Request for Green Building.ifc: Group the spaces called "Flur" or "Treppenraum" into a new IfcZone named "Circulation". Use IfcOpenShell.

First a look at what the model holds.

```python
import ifcopenshell

model = ifcopenshell.open("Green Building.ifc")
print(model.schema)
seen = {}
for space in model.by_type("IfcSpace"):
    seen[space.LongName] = seen.get(space.LongName, 0) + 1
for name, count in sorted(seen.items(), key=str):
    print(count, "x", name)
print("zones:", [z.Name for z in model.by_type("IfcZone")][:20])
```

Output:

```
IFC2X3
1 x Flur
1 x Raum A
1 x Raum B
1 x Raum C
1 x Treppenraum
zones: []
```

```python
import ifcopenshell
import ifcopenshell.api.group
import ifcopenshell.api.root

model = ifcopenshell.open("Green Building.ifc")

names = {"Flur", "Treppenraum"}
spaces = [s for s in model.by_type("IfcSpace") if s.LongName in names]

zone = ifcopenshell.api.root.create_entity(model, ifc_class="IfcZone", name="Circulation")
ifcopenshell.api.group.assign_group(model, products=spaces, group=zone)
print(len(spaces), "spaces in", zone.Name)

model.write("Green Building_rev.ifc")
```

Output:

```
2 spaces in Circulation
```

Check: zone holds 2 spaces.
